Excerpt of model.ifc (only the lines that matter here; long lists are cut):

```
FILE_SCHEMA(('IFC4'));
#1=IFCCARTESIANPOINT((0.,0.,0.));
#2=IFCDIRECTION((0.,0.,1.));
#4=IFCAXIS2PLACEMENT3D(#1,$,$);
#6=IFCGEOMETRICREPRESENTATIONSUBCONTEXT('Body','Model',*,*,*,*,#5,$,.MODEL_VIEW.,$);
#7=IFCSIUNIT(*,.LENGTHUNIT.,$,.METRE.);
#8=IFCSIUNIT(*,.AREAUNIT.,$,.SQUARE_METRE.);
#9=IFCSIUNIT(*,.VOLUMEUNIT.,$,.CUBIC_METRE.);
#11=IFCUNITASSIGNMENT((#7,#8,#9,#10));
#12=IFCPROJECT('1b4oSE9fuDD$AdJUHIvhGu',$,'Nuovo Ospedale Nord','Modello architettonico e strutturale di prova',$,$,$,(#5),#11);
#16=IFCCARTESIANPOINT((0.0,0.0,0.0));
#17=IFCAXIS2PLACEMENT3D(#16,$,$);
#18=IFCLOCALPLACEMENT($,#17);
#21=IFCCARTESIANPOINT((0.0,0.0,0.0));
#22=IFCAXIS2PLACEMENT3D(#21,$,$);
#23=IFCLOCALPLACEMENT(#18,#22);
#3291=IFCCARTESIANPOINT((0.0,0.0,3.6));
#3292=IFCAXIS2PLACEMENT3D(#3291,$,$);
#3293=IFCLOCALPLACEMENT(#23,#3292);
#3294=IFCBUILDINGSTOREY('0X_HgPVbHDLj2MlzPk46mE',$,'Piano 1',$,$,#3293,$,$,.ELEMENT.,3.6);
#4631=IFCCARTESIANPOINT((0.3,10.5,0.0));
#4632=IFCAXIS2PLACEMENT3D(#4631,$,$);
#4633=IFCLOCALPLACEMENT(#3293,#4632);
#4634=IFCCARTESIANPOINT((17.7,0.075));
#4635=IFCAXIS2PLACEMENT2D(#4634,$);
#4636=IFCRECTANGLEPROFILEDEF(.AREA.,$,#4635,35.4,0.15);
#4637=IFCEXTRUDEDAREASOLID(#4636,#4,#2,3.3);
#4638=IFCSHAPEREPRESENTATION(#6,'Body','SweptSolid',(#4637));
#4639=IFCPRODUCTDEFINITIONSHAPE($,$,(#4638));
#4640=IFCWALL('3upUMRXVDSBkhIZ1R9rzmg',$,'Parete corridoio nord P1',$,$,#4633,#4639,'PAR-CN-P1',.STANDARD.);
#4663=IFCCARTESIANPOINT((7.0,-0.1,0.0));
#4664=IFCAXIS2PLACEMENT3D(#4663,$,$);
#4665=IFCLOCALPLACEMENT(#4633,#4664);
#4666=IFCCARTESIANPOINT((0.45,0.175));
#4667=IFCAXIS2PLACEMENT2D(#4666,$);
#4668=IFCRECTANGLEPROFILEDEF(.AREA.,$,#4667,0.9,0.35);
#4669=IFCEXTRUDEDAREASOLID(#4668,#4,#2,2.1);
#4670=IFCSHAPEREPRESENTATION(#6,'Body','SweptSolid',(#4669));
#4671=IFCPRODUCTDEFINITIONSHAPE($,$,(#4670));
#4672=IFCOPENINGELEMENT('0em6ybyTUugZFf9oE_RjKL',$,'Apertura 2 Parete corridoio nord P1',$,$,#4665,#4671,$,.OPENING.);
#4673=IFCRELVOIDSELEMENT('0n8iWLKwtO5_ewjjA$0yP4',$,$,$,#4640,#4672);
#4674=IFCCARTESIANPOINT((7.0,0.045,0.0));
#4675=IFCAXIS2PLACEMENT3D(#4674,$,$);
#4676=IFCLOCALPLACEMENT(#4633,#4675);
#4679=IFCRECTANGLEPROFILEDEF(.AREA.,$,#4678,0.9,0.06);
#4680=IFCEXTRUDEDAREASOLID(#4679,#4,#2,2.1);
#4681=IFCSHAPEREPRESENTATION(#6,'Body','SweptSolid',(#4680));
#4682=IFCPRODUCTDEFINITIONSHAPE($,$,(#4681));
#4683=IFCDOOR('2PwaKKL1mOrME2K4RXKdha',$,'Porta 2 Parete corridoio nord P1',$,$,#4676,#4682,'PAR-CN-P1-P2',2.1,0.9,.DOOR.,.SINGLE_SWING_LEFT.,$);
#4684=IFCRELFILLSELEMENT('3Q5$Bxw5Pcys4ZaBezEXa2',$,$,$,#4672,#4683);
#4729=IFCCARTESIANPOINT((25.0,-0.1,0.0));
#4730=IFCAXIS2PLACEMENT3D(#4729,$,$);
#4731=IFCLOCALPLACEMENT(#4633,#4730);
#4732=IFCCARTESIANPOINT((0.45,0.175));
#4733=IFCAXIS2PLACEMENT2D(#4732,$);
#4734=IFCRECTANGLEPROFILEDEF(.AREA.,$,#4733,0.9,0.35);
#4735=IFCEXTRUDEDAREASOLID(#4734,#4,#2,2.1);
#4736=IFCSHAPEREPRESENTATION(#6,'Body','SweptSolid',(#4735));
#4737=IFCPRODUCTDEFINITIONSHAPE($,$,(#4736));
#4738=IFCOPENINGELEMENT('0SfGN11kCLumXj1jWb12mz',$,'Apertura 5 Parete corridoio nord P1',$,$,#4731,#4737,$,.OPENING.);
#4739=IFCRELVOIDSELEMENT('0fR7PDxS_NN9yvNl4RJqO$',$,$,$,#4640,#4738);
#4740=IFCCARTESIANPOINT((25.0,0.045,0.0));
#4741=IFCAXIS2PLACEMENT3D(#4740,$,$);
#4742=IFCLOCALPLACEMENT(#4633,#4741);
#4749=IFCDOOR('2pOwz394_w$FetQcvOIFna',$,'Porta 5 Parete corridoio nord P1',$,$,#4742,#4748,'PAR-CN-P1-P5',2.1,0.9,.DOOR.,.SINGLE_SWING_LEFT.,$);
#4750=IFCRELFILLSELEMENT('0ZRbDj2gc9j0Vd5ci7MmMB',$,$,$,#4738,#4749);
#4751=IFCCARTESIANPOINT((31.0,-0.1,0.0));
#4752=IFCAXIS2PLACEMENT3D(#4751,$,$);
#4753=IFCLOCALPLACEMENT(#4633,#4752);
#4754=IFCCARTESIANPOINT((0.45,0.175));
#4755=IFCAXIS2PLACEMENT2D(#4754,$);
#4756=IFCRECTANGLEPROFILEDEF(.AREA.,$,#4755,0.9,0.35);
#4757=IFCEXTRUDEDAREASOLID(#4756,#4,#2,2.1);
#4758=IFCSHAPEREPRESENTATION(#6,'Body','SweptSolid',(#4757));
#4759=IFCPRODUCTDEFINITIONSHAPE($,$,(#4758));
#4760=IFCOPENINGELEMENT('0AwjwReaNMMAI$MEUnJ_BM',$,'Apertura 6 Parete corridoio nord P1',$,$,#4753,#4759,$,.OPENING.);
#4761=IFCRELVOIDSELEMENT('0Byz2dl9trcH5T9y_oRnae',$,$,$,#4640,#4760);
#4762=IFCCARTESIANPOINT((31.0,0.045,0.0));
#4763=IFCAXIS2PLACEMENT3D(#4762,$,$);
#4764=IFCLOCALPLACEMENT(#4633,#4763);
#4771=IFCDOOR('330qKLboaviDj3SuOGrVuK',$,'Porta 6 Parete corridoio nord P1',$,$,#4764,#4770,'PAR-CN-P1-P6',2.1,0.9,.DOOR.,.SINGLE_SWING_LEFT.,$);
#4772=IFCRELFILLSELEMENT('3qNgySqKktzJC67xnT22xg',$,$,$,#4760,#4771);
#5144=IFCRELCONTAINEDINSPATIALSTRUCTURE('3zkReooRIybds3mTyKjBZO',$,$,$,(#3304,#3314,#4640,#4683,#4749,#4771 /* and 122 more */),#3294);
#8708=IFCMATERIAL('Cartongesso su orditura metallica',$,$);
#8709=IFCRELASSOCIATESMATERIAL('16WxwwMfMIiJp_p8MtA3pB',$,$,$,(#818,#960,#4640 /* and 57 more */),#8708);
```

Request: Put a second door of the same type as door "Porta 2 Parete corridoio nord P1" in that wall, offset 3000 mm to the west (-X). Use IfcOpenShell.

```python
import ifcopenshell
import ifcopenshell.api.feature
import ifcopenshell.api.geometry
import ifcopenshell.api.root
import ifcopenshell.geom
import ifcopenshell.util.element
import ifcopenshell.util.placement
import ifcopenshell.util.shape

model = ifcopenshell.open("model.ifc")
settings = ifcopenshell.geom.settings()


def volume(element):
    """Net volume in cubic metres, openings subtracted."""
    shape = ifcopenshell.geom.create_shape(settings, element)
    return ifcopenshell.util.shape.get_volume(shape.geometry)


door = model.by_id(4683)
opening = door.FillsVoids[0].RelatingOpeningElement
wall = opening.VoidsElements[0].RelatingBuildingElement
before = volume(wall)
shift = ifcopenshell.util.placement.get_local_placement(wall.ObjectPlacement)[:3, 0] * -3.0

# copy_class copies the void relationship, type, container and properties, but no geometry.
new_opening = ifcopenshell.api.root.copy_class(model, product=opening)
new_opening.Representation = ifcopenshell.util.element.copy_deep(
    model, opening.Representation, exclude=["IfcGeometricRepresentationContext", "IfcRepresentationMap"]
)
new_door = ifcopenshell.api.root.copy_class(model, product=door)
new_door.Representation = ifcopenshell.util.element.copy_deep(
    model, door.Representation, exclude=["IfcGeometricRepresentationContext", "IfcRepresentationMap"]
)
new_door.Tag = None
ifcopenshell.api.feature.add_filling(model, opening=new_opening, element=new_door)

for old, new in ((opening, new_opening), (door, new_door)):
    matrix = ifcopenshell.util.placement.get_local_placement(old.ObjectPlacement)
    matrix[:3, 3] += shift
    ifcopenshell.api.geometry.edit_object_placement(model, product=new, matrix=matrix, is_si=False)

after = volume(wall)

print(f"wall volume {before:.3f} -> {after:.3f} m3")

model.write("model-out.ifc")
```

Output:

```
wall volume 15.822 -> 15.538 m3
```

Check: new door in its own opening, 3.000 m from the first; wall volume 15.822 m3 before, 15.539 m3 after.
